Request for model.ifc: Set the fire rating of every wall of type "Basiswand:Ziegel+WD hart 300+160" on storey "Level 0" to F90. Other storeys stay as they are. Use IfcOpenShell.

First a look at what the model holds.

```python
import ifcopenshell
import ifcopenshell.util.element

model = ifcopenshell.open("model.ifc")
print(model.schema)
storey = next(s for s in model.by_type("IfcBuildingStorey") if s.Name == "Level 0")
walls = [e for e in ifcopenshell.util.element.get_decomposition(storey) if e.is_a("IfcWall")]
seen = {}
for e in walls:
    element_type = ifcopenshell.util.element.get_type(e)
    key = (element_type.Name if element_type != e and element_type else None, ifcopenshell.util.element.get_pset(e, "Pset_WallCommon", "FireRating"))
    seen[key] = seen.get(key, 0) + 1
for (name, value), count in sorted(seen.items(), key=str):
    print(count, "x", name, "|", value)
```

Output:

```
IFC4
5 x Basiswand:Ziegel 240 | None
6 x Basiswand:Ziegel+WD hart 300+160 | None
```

```python
import ifcopenshell
import ifcopenshell.api.pset
import ifcopenshell.util.element

model = ifcopenshell.open("model.ifc")

storey = next(s for s in model.by_type("IfcBuildingStorey") if s.Name == "Level 0")
walls = [e for e in ifcopenshell.util.element.get_decomposition(storey) if e.is_a("IfcWall")]

count = 0
for e in walls:
    element_type = ifcopenshell.util.element.get_type(e)
    if element_type in (None, e) or element_type.Name != "Basiswand:Ziegel+WD hart 300+160":
        continue
    # add_pset returns the element's existing set when there is one.
    pset = ifcopenshell.api.pset.add_pset(model, product=e, name="Pset_WallCommon")
    ifcopenshell.api.pset.edit_pset(model, pset=pset, properties={"FireRating": "F90"})
    count += 1

print(count, "walls updated")

model.write("model_edited.ifc")
```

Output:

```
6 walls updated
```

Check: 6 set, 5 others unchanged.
